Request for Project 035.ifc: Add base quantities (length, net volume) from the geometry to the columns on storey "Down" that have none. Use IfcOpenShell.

First a look at what the model holds.

```python
import ifcopenshell
import ifcopenshell.util.element
import ifcopenshell.util.unit

model = ifcopenshell.open("Project 035.ifc")
print(model.schema)
for unit_type in ("LENGTHUNIT", "AREAUNIT", "VOLUMEUNIT"):
    print(unit_type, ifcopenshell.util.unit.calculate_unit_scale(model, unit_type))
storey = next(s for s in model.by_type("IfcBuildingStorey") if s.Name == "Down")
columns = [e for e in ifcopenshell.util.element.get_decomposition(storey) if e.is_a("IfcColumn")]
for e in sorted(columns, key=lambda e: e.id()):
    print(e.id(), e.is_a(), e.Name, list(ifcopenshell.util.element.get_psets(e, qtos_only=True)), sep=" | ")
```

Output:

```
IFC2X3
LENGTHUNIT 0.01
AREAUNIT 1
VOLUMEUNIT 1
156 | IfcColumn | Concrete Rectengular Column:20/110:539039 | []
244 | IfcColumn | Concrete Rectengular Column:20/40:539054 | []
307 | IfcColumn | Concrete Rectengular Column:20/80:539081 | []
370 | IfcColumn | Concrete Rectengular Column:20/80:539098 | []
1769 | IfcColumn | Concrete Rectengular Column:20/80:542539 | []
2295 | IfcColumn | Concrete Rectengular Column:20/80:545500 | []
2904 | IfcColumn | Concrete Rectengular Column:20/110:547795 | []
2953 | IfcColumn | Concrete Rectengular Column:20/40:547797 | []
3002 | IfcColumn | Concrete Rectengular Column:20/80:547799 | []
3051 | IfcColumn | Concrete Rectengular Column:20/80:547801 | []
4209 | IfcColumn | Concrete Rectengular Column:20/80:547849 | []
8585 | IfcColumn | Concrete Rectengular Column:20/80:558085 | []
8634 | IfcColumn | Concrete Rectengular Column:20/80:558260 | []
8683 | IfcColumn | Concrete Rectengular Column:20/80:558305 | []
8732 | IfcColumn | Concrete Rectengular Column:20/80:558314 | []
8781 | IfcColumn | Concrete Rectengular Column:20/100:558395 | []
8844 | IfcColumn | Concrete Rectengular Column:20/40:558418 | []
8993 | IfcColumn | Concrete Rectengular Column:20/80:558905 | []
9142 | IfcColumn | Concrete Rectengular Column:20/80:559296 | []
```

```python
import ifcopenshell
import ifcopenshell.api.pset
import ifcopenshell.geom
import ifcopenshell.util.element
import ifcopenshell.util.shape
import ifcopenshell.util.unit

model = ifcopenshell.open("Project 035.ifc")
unit_scale = ifcopenshell.util.unit.calculate_unit_scale(model)
volume_scale = ifcopenshell.util.unit.calculate_unit_scale(model, "VOLUMEUNIT")
settings = ifcopenshell.geom.settings()

storey = next(s for s in model.by_type("IfcBuildingStorey") if s.Name == "Down")
columns = [e for e in ifcopenshell.util.element.get_decomposition(storey) if e.is_a("IfcColumn")]

for e in sorted(columns, key=lambda e: e.id()):
    if ifcopenshell.util.element.get_psets(e, qtos_only=True, should_inherit=False):
        continue
    # Geometry comes back in metres, in the element's own axes.
    shape = ifcopenshell.geom.create_shape(settings, e)
    values = {
        "Length": ifcopenshell.util.shape.get_z(shape.geometry) / unit_scale,
        "NetVolume": ifcopenshell.util.shape.get_volume(shape.geometry) / volume_scale,
    }
    qto = ifcopenshell.api.pset.add_qto(model, product=e, name="BaseQuantities")
    ifcopenshell.api.pset.edit_qto(model, qto=qto, properties=values)
    print(e.id(), {k: round(v, 3) for k, v in values.items()})

model.write("Project 035_rev.ifc")
```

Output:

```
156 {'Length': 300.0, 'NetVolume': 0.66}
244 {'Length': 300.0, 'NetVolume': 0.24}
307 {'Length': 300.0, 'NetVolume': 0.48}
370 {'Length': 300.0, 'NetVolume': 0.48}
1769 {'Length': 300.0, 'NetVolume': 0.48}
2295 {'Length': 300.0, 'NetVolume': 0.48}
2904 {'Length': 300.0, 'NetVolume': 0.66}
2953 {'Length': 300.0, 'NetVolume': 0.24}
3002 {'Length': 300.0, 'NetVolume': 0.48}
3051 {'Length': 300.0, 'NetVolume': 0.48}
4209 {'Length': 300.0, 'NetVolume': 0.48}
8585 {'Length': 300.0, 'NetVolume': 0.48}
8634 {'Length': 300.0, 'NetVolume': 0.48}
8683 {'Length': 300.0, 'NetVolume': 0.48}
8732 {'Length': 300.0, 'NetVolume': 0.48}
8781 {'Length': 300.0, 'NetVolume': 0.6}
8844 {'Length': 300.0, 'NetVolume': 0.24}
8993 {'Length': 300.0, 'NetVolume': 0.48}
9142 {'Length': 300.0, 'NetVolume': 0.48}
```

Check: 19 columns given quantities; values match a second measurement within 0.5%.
